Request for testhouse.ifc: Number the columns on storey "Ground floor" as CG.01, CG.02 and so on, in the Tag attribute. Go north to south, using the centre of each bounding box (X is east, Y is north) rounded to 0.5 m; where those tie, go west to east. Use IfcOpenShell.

First a look at what the model holds.

```python
import ifcopenshell
import ifcopenshell.util.element
import ifcopenshell.util.placement

model = ifcopenshell.open("testhouse.ifc")
print(model.schema)
storey = next(s for s in model.by_type("IfcBuildingStorey") if s.Name == "Ground floor")
columns = [e for e in ifcopenshell.util.element.get_decomposition(storey) if e.is_a("IfcColumn")]
for e in sorted(columns, key=lambda e: e.id()):
    origin = ifcopenshell.util.placement.get_local_placement(e.ObjectPlacement)[:3, 3]
    print(e.id(), e.Tag, e.Name, origin.round(2) + 0.0, sep=" | ")
```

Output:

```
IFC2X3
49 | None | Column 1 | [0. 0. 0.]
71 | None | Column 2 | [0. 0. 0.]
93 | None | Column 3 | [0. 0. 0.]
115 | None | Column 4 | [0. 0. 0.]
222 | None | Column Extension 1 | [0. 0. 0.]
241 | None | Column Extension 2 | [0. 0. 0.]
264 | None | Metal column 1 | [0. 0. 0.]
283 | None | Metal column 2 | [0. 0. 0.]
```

```python
import ifcopenshell
import ifcopenshell.geom
import ifcopenshell.util.element
import ifcopenshell.util.shape

model = ifcopenshell.open("testhouse.ifc")
settings = ifcopenshell.geom.settings()
settings.set("use-world-coords", True)


def centre(element):
    shape = ifcopenshell.geom.create_shape(settings, element)
    return ifcopenshell.util.shape.get_bbox_centroid(shape.geometry)


storey = next(s for s in model.by_type("IfcBuildingStorey") if s.Name == "Ground floor")
columns = [e for e in ifcopenshell.util.element.get_decomposition(storey) if e.is_a("IfcColumn")]

# Insertion points can sit at a corner or the storey origin, so sort by the geometry (in metres).
centres = {e: centre(e) for e in columns}
columns.sort(key=lambda e: (-round(centres[e][1] / 0.5), centres[e][0]))

for i, e in enumerate(columns, start=1):
    number = f"CG.{i:02d}"
    e.Tag = number
    print(e.id(), number)

model.write("testhouse_edited.ifc")
```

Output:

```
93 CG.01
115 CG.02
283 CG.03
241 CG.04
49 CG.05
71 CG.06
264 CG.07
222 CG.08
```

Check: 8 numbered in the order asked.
